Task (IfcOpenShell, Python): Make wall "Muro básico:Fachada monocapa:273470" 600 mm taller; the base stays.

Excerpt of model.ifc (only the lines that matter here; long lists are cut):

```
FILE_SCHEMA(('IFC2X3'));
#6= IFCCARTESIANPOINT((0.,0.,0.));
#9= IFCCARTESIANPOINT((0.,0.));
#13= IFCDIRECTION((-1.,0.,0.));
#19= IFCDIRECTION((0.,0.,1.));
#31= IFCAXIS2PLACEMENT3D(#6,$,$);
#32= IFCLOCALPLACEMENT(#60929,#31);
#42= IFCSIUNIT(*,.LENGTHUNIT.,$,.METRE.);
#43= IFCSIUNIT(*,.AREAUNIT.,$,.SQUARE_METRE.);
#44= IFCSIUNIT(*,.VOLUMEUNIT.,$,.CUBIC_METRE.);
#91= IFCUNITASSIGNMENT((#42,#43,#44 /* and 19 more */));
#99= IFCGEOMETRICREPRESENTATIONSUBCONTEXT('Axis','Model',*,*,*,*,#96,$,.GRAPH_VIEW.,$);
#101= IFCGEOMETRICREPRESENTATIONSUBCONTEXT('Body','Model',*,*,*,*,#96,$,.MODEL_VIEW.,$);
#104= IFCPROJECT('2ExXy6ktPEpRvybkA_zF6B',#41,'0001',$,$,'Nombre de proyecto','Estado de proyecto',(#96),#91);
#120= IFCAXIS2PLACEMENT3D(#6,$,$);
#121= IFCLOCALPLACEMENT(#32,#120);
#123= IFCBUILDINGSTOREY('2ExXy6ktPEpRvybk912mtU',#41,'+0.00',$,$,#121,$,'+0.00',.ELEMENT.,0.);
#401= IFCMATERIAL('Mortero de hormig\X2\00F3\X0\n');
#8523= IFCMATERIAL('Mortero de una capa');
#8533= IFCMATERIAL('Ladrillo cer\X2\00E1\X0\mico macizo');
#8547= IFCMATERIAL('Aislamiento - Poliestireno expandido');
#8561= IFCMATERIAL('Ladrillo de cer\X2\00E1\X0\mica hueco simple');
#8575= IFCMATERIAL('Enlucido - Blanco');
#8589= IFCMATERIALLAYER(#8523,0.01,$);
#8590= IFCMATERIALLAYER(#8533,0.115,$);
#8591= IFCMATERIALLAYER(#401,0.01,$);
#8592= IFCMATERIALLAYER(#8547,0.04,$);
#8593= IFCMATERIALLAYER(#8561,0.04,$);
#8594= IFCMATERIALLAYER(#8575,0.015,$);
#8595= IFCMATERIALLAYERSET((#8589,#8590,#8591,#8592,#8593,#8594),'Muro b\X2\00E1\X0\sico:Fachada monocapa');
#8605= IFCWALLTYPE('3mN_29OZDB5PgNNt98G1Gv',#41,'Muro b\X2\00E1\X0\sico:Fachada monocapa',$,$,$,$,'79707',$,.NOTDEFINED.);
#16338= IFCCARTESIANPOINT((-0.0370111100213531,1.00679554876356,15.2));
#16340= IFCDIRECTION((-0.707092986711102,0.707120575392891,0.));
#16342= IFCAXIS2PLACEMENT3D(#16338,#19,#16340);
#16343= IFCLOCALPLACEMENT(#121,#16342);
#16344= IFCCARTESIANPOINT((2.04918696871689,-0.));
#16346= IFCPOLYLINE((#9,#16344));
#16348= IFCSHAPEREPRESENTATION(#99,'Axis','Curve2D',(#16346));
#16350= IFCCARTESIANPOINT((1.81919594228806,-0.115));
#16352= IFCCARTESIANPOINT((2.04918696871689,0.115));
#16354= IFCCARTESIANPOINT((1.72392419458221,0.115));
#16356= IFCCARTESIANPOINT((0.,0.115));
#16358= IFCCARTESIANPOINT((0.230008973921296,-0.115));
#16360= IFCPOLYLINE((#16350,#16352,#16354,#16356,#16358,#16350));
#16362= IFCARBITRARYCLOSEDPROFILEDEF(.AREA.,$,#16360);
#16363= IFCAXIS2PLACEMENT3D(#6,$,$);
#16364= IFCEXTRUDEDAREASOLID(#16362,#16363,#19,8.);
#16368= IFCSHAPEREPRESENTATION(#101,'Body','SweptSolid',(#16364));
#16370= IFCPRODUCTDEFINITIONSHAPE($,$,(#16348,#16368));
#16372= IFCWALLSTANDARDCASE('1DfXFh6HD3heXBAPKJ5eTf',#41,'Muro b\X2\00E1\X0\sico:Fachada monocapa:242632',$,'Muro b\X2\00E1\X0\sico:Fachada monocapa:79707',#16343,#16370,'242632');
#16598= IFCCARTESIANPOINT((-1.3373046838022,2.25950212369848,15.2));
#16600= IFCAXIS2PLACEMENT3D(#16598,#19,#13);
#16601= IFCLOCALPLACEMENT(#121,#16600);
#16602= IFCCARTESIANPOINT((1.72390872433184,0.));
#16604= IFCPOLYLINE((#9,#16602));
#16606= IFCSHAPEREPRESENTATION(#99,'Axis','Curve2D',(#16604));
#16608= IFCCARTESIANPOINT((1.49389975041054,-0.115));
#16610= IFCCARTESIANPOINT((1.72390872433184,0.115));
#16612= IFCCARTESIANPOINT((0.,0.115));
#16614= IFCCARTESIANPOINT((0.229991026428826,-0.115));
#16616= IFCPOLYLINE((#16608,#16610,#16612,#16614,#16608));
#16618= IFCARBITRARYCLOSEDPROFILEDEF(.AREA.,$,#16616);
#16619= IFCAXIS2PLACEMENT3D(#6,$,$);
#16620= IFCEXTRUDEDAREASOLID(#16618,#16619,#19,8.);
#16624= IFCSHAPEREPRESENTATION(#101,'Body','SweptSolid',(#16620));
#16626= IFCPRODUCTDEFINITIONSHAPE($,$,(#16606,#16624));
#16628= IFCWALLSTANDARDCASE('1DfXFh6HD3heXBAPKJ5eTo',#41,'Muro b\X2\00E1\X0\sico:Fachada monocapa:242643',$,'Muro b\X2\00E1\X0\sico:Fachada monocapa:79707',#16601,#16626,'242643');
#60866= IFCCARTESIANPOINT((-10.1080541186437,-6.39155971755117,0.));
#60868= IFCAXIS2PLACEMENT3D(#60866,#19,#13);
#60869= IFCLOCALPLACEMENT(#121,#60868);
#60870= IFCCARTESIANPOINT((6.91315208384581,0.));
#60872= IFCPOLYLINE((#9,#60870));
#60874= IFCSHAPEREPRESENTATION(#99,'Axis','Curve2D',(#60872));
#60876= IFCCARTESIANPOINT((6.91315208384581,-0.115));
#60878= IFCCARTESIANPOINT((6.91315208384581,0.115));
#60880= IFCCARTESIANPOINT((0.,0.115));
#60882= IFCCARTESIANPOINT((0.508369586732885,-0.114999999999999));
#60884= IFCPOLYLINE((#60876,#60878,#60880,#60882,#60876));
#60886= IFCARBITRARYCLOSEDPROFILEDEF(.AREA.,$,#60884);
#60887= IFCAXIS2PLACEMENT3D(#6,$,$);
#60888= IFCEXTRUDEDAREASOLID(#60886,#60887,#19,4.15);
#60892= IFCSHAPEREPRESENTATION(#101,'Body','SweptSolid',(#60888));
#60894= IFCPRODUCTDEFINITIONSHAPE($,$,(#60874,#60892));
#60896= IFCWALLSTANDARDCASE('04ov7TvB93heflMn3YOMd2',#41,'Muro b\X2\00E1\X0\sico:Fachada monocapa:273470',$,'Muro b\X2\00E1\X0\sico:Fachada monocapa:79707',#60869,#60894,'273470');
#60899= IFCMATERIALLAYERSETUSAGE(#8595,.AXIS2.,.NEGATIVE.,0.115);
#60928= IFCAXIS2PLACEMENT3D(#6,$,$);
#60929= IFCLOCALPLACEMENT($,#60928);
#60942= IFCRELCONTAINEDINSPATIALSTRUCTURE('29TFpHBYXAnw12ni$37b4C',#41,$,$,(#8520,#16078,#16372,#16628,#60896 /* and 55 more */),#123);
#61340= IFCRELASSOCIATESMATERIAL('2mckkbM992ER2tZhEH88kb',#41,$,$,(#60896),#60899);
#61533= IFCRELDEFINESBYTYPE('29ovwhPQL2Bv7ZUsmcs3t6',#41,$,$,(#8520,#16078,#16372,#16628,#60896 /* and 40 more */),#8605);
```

```python
import ifcopenshell
import ifcopenshell.geom
import ifcopenshell.util.representation
import ifcopenshell.util.shape
import ifcopenshell.util.unit

model = ifcopenshell.open("model.ifc")
unit_scale = ifcopenshell.util.unit.calculate_unit_scale(model)
settings = ifcopenshell.geom.settings()


def volume(element):
    """Net volume in cubic metres, openings subtracted."""
    shape = ifcopenshell.geom.create_shape(settings, element)
    return ifcopenshell.util.shape.get_volume(shape.geometry)


wall = model.by_guid("04ov7TvB93heflMn3YOMd2")
before = volume(wall)

body = ifcopenshell.util.representation.get_representation(wall, "Model", "Body")
solid = body.Items[0]
old_height = solid.Depth
solid.Depth += 0.6 / unit_scale
after = volume(wall)

print(f"height {old_height:g} -> {solid.Depth:g}, volume {before:.3f} -> {after:.3f} m3")

model.write("model_updated.ifc")
```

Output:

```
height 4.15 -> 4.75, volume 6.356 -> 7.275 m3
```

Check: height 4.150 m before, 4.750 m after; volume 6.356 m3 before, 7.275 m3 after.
